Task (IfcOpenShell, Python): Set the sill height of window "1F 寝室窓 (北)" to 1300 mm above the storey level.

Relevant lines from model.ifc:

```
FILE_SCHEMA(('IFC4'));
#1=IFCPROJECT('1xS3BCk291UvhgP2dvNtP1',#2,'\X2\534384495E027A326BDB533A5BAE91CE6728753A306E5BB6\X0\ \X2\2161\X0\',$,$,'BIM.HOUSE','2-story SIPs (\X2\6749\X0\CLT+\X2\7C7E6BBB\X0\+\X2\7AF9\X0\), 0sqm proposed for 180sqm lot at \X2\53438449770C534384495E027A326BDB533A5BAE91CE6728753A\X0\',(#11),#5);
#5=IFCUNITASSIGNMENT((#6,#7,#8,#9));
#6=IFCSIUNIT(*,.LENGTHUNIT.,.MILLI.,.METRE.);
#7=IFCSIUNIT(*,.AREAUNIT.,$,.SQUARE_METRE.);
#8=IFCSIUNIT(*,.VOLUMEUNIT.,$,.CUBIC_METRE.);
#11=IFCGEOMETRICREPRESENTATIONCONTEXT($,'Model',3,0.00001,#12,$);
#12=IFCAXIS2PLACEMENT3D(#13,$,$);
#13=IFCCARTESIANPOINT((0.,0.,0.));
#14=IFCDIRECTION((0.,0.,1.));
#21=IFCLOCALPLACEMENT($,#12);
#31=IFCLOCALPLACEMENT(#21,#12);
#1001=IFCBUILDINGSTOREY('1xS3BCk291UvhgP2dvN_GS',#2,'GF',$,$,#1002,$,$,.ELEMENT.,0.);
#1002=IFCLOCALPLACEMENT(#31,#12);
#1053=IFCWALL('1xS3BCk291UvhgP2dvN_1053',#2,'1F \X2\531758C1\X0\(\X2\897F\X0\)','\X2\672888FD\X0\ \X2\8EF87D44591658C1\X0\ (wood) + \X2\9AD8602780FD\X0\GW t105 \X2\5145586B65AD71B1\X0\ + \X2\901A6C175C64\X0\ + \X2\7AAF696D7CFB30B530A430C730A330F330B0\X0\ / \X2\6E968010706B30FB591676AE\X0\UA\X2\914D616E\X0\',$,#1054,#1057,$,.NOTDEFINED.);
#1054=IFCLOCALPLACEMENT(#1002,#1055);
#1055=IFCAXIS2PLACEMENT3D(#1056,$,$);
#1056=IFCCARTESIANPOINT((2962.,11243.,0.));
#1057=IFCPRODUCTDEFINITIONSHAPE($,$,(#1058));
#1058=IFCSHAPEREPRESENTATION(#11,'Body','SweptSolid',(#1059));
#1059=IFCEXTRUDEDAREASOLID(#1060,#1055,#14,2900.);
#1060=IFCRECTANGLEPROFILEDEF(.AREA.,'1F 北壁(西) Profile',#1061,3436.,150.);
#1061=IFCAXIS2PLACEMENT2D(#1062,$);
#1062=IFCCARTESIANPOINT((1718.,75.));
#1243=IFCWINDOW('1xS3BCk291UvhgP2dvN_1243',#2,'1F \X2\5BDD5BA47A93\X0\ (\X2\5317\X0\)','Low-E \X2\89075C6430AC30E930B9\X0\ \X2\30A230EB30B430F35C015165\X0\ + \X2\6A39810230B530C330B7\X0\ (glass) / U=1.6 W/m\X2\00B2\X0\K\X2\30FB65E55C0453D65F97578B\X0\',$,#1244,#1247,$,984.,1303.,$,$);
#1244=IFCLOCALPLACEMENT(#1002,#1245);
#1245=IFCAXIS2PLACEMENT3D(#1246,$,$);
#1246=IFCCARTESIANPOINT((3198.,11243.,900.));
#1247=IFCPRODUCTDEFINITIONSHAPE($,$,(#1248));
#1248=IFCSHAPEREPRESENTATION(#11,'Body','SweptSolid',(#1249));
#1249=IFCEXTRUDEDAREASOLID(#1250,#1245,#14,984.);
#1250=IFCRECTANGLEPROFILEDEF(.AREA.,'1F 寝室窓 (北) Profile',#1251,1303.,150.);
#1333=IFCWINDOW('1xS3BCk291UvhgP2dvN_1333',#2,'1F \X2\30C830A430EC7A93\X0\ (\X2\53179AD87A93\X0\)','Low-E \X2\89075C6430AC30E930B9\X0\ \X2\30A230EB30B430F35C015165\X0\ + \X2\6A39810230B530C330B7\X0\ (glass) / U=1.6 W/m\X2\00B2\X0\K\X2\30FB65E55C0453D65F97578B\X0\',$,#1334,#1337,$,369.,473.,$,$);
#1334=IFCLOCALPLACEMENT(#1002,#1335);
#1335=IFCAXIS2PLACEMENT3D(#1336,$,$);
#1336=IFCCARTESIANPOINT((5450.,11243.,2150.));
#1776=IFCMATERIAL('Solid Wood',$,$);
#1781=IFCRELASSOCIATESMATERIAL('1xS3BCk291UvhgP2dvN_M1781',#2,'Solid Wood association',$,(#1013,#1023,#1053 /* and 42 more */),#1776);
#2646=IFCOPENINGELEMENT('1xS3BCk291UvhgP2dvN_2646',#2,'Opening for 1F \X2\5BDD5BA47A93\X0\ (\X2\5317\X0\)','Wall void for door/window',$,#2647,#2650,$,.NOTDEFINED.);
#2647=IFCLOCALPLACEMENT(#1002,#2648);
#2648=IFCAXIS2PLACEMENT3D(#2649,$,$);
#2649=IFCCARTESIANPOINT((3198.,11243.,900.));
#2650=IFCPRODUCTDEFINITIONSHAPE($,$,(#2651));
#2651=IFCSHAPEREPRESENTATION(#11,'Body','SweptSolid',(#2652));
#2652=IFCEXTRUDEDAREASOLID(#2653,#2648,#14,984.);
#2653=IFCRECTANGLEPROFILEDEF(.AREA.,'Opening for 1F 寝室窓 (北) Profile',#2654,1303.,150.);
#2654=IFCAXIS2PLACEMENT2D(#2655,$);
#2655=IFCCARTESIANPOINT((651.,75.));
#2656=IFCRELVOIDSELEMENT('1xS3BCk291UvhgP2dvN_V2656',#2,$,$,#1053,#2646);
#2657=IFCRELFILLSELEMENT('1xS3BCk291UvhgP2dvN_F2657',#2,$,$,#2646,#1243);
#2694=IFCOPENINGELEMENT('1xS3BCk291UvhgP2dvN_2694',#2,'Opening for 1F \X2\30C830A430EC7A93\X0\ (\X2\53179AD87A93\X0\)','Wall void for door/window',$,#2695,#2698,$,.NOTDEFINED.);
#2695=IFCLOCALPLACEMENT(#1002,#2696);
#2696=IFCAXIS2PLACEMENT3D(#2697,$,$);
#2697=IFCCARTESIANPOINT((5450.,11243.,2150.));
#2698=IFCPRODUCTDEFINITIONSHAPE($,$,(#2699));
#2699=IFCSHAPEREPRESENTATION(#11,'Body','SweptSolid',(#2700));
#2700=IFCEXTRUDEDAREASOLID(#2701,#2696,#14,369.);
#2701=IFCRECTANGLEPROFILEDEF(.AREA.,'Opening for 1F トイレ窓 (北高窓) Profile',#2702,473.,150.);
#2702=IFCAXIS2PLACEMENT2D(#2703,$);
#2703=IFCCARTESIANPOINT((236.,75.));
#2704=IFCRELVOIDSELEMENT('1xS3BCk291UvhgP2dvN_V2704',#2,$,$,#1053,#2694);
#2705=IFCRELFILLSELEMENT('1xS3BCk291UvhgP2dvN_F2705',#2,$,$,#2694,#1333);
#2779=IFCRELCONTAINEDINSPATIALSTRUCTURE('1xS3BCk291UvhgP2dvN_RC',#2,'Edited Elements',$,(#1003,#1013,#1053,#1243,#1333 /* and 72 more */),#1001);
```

```python
import numpy as np
import ifcopenshell
import ifcopenshell.api.geometry
import ifcopenshell.geom
import ifcopenshell.util.element
import ifcopenshell.util.placement
import ifcopenshell.util.shape
import ifcopenshell.util.unit

model = ifcopenshell.open("model.ifc")
unit_scale = ifcopenshell.util.unit.calculate_unit_scale(model)

window = model.by_guid("1xS3BCk291UvhgP2dvN_1243")
opening = window.FillsVoids[0].RelatingOpeningElement
storey = ifcopenshell.util.element.get_container(window, ifc_class="IfcBuildingStorey")
level = ifcopenshell.util.placement.get_local_placement(storey.ObjectPlacement)[2, 3]

# The opening's origin need not be at the sill, so measure its lowest point.
shape = ifcopenshell.geom.create_shape(ifcopenshell.geom.settings(), opening)
bottom = ifcopenshell.util.shape.get_shape_bottom_elevation(shape, shape.geometry) / unit_scale
dz = level + 1.3 / unit_scale - bottom

shift = np.array([0.0, 0.0, dz])
# The window is not placed relative to its opening, so move both.
for product in (opening, window):
    matrix = ifcopenshell.util.placement.get_local_placement(product.ObjectPlacement)
    matrix[:3, 3] += shift
    ifcopenshell.api.geometry.edit_object_placement(model, product=product, matrix=matrix, is_si=False)

print(f"moved by {dz * unit_scale:+.3f} m")

model.write("model_v2.ifc")
```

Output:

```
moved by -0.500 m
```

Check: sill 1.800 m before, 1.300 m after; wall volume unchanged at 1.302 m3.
